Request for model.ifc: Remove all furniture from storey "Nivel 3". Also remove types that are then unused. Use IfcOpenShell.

First a look at what the model holds.

```python
import ifcopenshell
import ifcopenshell.util.element

model = ifcopenshell.open("model.ifc")
print(model.schema)
storey = next(s for s in model.by_type("IfcBuildingStorey") if s.Name == "Nivel 3")
furniture = [e for e in ifcopenshell.util.element.get_decomposition(storey) if e.is_a("IfcFurnishingElement")]
seen = {}
for e in furniture:
    element_type = ifcopenshell.util.element.get_type(e)
    name = element_type.Name if element_type not in (None, e) else None
    seen[name] = seen.get(name, 0) + 1
for name, count in sorted(seen.items(), key=str):
    print(count, "x", name)
```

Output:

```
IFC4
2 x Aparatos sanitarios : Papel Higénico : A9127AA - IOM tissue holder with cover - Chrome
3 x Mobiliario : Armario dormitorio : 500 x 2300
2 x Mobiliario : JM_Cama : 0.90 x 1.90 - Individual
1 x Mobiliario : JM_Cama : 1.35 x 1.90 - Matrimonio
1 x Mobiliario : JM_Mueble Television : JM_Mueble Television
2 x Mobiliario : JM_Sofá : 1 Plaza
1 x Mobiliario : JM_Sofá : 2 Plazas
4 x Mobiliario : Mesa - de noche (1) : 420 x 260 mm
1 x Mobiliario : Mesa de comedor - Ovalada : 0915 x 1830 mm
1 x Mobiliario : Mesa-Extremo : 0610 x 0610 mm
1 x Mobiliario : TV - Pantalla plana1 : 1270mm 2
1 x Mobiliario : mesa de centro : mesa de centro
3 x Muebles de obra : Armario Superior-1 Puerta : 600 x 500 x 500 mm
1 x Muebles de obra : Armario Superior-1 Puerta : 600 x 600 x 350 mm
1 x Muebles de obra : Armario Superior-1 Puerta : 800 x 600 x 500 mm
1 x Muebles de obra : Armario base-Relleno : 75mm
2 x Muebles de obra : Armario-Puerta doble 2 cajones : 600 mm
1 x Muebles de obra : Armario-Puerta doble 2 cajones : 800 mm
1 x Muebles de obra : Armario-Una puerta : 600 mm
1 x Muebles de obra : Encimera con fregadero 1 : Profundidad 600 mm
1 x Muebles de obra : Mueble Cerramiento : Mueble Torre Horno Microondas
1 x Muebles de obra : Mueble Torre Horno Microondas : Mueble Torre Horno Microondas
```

```python
import ifcopenshell
import ifcopenshell.api.root
import ifcopenshell.util.element

model = ifcopenshell.open("model.ifc")

storey = next(s for s in model.by_type("IfcBuildingStorey") if s.Name == "Nivel 3")
furniture = [e for e in ifcopenshell.util.element.get_decomposition(storey) if e.is_a("IfcFurnishingElement")]
types = {ifcopenshell.util.element.get_type(e) for e in furniture} - {None, *furniture}

for e in furniture:
    ifcopenshell.api.root.remove_product(model, product=e)
print(len(furniture), "removed")

unused = [t for t in types if not ifcopenshell.util.element.get_types(t)]
for t in unused:
    ifcopenshell.api.root.remove_product(model, product=t)
print(len(unused), "unused types removed")

model.write("model-out.ifc")
```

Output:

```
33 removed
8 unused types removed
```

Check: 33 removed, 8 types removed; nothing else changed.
